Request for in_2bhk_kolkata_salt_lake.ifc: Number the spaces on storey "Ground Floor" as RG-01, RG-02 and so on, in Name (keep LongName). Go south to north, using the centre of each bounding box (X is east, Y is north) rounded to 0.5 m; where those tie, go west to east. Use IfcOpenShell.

First a look at what the model holds.

```python
import ifcopenshell
import ifcopenshell.util.element
import ifcopenshell.util.placement

model = ifcopenshell.open("in_2bhk_kolkata_salt_lake.ifc")
print(model.schema)
storey = next(s for s in model.by_type("IfcBuildingStorey") if s.Name == "Ground Floor")
spaces = [e for e in ifcopenshell.util.element.get_decomposition(storey) if e.is_a("IfcSpace")]
for e in sorted(spaces, key=lambda e: e.id()):
    origin = ifcopenshell.util.placement.get_local_placement(e.ObjectPlacement)[:3, 3]
    print(e.id(), e.Name, e.LongName, origin.round(2) + 0.0, sep=" | ")
```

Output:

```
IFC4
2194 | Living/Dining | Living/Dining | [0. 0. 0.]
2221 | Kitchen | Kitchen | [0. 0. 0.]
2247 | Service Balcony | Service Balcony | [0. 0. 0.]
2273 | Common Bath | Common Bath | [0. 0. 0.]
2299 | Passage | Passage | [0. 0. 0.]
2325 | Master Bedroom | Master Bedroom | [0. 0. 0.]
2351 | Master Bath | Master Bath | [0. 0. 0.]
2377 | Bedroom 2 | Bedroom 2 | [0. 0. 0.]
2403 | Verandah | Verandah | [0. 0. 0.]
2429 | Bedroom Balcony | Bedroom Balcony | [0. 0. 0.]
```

```python
import ifcopenshell
import ifcopenshell.geom
import ifcopenshell.util.element
import ifcopenshell.util.shape

model = ifcopenshell.open("in_2bhk_kolkata_salt_lake.ifc")
settings = ifcopenshell.geom.settings()
settings.set("use-world-coords", True)


def centre(element):
    shape = ifcopenshell.geom.create_shape(settings, element)
    return ifcopenshell.util.shape.get_bbox_centroid(shape.geometry)


storey = next(s for s in model.by_type("IfcBuildingStorey") if s.Name == "Ground Floor")
spaces = [e for e in ifcopenshell.util.element.get_decomposition(storey) if e.is_a("IfcSpace")]

# Insertion points can sit at a corner or the storey origin, so sort by the geometry (in metres).
centres = {e: centre(e) for e in spaces}
spaces.sort(key=lambda e: (round(centres[e][1] / 0.5), centres[e][0]))

for i, e in enumerate(spaces, start=1):
    number = f"RG-{i:02d}"
    e.Name = number
    print(e.id(), number)

model.write("in_2bhk_kolkata_salt_lake_v2.ifc")
```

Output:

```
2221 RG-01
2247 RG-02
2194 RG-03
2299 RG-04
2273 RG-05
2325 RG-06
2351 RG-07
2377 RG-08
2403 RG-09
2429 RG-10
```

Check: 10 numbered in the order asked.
